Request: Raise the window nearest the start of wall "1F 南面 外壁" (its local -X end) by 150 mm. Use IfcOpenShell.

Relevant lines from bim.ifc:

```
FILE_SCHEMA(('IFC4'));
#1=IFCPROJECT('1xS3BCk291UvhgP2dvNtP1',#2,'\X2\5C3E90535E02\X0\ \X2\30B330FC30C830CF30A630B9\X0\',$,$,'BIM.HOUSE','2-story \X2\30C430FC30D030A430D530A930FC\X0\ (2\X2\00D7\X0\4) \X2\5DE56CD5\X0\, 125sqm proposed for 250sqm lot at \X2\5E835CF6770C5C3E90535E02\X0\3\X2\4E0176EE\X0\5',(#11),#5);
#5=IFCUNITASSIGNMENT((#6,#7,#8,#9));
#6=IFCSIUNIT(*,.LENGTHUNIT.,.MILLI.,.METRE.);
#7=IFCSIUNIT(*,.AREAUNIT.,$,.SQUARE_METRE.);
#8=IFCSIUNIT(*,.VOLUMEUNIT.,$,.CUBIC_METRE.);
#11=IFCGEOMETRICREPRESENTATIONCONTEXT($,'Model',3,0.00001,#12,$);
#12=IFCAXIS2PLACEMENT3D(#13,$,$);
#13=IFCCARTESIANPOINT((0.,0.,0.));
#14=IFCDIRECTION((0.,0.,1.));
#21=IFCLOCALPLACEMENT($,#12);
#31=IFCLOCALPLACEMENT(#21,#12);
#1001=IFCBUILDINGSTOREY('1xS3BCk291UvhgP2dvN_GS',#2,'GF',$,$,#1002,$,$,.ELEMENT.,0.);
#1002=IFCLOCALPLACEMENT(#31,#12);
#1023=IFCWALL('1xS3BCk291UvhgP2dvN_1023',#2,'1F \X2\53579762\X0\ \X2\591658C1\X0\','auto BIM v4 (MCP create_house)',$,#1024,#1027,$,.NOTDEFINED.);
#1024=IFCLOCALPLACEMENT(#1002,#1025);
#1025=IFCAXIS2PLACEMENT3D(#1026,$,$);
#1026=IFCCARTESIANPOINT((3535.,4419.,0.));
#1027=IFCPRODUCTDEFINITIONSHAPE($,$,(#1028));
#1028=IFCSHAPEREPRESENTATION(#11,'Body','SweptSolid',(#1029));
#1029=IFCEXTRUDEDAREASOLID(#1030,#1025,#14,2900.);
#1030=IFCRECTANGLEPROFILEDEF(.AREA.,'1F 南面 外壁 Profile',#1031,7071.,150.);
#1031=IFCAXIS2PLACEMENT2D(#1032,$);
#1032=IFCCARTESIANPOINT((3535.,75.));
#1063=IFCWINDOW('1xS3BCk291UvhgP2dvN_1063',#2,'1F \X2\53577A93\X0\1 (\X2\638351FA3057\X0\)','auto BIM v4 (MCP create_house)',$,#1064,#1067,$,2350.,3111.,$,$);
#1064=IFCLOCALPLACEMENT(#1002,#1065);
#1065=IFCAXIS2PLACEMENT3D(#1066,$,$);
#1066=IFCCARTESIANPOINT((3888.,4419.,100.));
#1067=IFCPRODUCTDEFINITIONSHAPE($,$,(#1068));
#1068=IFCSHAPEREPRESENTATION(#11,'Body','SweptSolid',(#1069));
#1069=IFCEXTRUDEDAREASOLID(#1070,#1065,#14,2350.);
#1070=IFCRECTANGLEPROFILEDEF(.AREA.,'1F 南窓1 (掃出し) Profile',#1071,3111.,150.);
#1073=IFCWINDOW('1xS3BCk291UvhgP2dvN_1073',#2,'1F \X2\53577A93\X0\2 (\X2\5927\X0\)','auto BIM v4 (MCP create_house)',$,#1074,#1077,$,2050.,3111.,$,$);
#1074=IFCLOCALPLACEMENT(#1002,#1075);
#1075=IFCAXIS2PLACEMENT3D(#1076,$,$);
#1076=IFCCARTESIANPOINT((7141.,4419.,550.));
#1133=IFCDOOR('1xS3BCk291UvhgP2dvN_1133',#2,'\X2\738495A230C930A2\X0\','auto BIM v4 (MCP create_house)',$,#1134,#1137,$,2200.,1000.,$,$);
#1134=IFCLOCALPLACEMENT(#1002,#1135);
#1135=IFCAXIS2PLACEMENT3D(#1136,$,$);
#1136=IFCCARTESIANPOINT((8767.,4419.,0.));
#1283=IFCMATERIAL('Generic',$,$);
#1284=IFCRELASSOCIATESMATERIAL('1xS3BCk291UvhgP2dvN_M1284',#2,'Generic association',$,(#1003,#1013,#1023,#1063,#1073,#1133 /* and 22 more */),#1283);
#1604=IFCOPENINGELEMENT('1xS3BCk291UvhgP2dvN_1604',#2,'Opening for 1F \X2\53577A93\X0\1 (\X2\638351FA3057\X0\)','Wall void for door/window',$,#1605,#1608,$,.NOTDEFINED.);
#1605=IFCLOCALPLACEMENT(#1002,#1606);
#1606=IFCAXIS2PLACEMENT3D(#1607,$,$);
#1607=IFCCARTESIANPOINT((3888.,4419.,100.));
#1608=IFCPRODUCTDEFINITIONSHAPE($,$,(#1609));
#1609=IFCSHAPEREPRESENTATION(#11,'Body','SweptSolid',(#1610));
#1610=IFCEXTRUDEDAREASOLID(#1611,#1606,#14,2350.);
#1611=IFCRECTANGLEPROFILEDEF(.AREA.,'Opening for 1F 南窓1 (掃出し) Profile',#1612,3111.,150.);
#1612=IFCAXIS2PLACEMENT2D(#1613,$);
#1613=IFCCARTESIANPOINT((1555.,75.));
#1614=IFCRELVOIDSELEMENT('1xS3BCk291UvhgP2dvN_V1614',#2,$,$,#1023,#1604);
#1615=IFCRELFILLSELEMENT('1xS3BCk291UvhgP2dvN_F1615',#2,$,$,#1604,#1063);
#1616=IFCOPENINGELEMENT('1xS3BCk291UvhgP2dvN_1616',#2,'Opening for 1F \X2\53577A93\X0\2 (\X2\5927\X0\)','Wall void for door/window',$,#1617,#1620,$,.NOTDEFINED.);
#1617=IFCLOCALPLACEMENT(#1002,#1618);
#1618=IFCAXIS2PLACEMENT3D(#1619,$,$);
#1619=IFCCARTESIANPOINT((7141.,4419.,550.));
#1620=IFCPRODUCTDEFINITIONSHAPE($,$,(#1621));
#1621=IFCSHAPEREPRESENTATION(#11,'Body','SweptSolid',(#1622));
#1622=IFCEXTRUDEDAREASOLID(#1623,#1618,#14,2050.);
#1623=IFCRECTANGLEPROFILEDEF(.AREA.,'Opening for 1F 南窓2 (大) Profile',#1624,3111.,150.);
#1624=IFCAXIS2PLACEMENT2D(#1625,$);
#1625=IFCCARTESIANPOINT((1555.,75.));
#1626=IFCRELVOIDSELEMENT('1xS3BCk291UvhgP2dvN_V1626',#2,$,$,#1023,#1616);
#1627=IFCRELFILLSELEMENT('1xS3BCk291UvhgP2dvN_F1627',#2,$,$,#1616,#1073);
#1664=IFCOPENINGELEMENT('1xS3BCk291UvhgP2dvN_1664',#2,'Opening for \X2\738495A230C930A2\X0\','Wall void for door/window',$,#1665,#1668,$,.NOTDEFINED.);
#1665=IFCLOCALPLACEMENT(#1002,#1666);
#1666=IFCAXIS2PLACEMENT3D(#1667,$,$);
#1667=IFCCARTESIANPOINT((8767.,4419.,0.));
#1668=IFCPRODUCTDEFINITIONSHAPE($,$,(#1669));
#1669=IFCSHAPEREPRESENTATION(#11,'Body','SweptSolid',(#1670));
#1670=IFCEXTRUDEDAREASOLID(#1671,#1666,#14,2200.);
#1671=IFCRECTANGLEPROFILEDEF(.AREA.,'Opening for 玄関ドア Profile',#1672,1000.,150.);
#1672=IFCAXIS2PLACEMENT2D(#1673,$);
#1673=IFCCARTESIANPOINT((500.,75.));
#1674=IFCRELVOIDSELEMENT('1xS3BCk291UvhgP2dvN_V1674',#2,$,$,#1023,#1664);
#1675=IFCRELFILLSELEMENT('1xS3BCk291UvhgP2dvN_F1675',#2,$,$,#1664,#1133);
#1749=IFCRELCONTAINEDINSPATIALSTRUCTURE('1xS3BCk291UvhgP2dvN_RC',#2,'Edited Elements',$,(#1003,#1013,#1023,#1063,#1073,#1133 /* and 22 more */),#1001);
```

```python
import numpy as np
import ifcopenshell
import ifcopenshell.api.geometry
import ifcopenshell.util.placement
import ifcopenshell.util.unit

model = ifcopenshell.open("bim.ifc")
unit_scale = ifcopenshell.util.unit.calculate_unit_scale(model)

window = model.by_guid("1xS3BCk291UvhgP2dvN_1063")
opening = window.FillsVoids[0].RelatingOpeningElement
dz = 150.0

shift = np.array([0.0, 0.0, dz])
# The window is not placed relative to its opening, so move both.
for product in (opening, window):
    matrix = ifcopenshell.util.placement.get_local_placement(product.ObjectPlacement)
    matrix[:3, 3] += shift
    ifcopenshell.api.geometry.edit_object_placement(model, product=product, matrix=matrix, is_si=False)

print(f"moved by {dz * unit_scale:+.3f} m")

model.write("bim-out.ifc")
```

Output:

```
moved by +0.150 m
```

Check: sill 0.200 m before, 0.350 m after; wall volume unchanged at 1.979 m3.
